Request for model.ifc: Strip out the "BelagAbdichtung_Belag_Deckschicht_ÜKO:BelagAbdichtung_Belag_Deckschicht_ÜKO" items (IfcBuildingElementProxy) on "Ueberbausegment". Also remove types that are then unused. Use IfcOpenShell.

First a look at what the model holds.

```python
import ifcopenshell
import ifcopenshell.util.element

model = ifcopenshell.open("model.ifc")
print(model.schema)
storey = next(s for s in model.by_type("IfcBuildingStorey") if s.Name == "Ueberbausegment")
proxies = [e for e in ifcopenshell.util.element.get_decomposition(storey) if e.is_a("IfcBuildingElementProxy")]
seen = {}
for e in proxies:
    element_type = ifcopenshell.util.element.get_type(e)
    name = element_type.Name if element_type not in (None, e) else None
    seen[name] = seen.get(name, 0) + 1
for name, count in sorted(seen.items(), key=str):
    print(count, "x", name)
```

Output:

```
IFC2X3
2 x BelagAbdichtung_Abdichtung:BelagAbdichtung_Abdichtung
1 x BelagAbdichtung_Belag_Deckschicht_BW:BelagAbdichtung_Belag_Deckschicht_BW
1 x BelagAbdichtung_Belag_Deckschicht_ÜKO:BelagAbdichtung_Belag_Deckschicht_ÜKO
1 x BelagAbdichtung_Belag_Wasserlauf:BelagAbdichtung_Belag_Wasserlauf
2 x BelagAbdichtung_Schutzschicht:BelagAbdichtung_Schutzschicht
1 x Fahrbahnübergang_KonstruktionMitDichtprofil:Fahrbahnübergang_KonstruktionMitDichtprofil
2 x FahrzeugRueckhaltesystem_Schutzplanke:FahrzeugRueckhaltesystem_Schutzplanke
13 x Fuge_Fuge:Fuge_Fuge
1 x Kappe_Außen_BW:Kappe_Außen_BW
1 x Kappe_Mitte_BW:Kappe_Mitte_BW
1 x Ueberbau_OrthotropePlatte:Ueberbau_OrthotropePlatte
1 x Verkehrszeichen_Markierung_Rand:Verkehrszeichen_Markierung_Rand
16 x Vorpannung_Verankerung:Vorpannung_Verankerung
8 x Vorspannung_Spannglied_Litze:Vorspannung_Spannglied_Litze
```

```python
import ifcopenshell
import ifcopenshell.api.root
import ifcopenshell.util.element

model = ifcopenshell.open("model.ifc")

storey = next(s for s in model.by_type("IfcBuildingStorey") if s.Name == "Ueberbausegment")
proxies = [e for e in ifcopenshell.util.element.get_decomposition(storey) if e.is_a("IfcBuildingElementProxy")]
targets = [e for e in proxies if (t := ifcopenshell.util.element.get_type(e)) not in (None, e) and t.Name == "BelagAbdichtung_Belag_Deckschicht_ÜKO:BelagAbdichtung_Belag_Deckschicht_ÜKO"]
types = {ifcopenshell.util.element.get_type(e) for e in targets} - {None, *targets}

for e in targets:
    ifcopenshell.api.root.remove_product(model, product=e)
print(len(targets), "removed")

unused = [t for t in types if not ifcopenshell.util.element.get_types(t)]
for t in unused:
    ifcopenshell.api.root.remove_product(model, product=t)
print(len(unused), "unused types removed")

model.write("model_updated.ifc")
```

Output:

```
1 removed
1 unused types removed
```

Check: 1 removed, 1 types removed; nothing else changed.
